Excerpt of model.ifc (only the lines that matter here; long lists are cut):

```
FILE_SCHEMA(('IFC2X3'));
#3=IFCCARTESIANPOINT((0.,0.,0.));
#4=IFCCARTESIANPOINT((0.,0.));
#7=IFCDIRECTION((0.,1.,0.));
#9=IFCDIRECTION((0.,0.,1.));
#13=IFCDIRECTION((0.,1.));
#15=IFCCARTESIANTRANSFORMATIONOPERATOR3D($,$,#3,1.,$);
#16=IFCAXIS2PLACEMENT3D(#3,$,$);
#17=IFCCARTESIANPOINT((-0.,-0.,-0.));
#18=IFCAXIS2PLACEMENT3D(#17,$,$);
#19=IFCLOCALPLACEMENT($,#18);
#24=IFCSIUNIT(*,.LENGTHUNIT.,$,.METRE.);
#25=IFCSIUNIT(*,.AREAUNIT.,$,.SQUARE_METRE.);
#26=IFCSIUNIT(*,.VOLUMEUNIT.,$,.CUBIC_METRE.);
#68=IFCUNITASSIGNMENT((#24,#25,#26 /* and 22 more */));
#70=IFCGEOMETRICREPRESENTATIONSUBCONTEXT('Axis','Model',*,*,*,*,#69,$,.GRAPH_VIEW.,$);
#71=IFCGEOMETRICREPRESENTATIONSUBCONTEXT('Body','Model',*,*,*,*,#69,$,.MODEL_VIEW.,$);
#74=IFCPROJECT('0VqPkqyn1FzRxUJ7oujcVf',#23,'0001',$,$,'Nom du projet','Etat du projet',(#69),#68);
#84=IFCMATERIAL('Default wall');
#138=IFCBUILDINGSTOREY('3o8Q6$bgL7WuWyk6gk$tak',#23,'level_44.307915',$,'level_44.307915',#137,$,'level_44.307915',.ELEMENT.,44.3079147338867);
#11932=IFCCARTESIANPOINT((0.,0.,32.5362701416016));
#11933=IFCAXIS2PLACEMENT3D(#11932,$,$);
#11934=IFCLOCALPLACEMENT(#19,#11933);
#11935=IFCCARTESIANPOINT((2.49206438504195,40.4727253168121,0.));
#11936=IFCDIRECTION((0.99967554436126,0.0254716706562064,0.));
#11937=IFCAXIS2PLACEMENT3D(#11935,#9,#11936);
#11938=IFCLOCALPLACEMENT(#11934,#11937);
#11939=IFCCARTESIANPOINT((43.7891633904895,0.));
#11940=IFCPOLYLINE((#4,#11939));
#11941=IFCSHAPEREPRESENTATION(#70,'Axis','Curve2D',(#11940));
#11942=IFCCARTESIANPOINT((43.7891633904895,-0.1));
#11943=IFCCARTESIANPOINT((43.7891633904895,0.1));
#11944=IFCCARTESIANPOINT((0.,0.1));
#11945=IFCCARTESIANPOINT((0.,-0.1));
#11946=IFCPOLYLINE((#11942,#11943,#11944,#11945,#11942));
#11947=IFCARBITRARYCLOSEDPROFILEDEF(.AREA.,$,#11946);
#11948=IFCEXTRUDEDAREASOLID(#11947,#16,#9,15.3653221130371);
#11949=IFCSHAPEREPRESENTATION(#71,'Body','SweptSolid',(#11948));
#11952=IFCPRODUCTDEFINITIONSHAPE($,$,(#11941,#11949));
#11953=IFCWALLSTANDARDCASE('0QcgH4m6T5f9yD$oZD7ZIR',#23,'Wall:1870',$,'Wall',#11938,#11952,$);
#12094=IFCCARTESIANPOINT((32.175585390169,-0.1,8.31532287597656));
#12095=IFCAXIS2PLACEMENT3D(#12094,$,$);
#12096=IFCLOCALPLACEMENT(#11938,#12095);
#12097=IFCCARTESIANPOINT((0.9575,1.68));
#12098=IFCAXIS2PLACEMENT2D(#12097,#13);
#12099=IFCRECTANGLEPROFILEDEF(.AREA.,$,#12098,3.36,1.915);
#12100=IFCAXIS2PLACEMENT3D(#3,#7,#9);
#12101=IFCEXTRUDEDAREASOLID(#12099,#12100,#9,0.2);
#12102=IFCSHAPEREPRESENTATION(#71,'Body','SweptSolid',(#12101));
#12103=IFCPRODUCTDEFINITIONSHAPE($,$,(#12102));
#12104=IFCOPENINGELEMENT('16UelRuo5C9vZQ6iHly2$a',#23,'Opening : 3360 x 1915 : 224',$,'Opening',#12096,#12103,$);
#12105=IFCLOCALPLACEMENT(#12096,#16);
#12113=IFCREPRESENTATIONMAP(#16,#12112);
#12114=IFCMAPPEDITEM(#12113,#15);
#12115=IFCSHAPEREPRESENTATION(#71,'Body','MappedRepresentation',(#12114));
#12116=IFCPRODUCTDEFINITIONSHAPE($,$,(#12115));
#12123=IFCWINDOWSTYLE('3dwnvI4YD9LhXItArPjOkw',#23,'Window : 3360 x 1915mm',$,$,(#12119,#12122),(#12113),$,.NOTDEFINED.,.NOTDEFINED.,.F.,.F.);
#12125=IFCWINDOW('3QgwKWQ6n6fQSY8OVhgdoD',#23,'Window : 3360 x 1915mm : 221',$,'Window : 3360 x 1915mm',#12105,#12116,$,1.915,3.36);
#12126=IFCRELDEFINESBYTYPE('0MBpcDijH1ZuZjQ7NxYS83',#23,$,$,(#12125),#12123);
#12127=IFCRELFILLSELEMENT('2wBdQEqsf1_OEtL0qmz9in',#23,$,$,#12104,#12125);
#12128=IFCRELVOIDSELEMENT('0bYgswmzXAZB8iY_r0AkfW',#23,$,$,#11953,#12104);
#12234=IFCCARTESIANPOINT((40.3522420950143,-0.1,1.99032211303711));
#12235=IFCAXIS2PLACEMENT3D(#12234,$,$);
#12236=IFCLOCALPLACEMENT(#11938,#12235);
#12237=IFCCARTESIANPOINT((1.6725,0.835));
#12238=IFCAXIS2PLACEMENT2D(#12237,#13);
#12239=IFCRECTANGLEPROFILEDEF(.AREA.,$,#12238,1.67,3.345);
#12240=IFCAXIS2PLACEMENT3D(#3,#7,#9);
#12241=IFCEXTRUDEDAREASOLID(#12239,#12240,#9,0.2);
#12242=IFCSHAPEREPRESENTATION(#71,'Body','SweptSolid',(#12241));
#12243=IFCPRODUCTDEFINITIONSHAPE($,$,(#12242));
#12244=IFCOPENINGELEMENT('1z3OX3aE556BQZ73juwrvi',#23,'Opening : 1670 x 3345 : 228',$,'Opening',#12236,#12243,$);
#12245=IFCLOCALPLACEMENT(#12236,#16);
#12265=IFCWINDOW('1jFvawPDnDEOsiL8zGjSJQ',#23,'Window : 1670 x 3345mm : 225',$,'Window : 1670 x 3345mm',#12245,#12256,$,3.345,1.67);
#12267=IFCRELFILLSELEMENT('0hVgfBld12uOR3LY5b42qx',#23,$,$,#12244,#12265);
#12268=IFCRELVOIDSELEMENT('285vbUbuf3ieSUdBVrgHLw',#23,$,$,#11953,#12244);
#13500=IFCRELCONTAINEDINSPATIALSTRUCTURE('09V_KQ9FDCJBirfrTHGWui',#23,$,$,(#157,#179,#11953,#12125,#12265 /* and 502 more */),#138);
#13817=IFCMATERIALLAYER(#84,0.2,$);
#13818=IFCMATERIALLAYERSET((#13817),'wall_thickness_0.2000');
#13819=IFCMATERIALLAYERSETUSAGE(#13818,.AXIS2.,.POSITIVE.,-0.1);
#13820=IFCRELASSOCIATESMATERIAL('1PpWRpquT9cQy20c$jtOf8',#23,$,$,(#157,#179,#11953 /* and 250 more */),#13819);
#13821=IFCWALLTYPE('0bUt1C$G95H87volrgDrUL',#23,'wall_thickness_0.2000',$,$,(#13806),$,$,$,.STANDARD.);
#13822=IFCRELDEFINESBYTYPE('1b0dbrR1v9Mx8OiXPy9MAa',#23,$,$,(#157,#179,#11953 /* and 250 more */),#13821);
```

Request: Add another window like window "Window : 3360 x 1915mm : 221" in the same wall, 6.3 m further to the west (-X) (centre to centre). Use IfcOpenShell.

```python
import ifcopenshell
import ifcopenshell.api.feature
import ifcopenshell.api.geometry
import ifcopenshell.api.root
import ifcopenshell.geom
import ifcopenshell.util.element
import ifcopenshell.util.placement
import ifcopenshell.util.shape

model = ifcopenshell.open("model.ifc")
settings = ifcopenshell.geom.settings()


def volume(element):
    """Net volume in cubic metres, openings subtracted."""
    shape = ifcopenshell.geom.create_shape(settings, element)
    return ifcopenshell.util.shape.get_volume(shape.geometry)


window = model.by_guid("3QgwKWQ6n6fQSY8OVhgdoD")
opening = window.FillsVoids[0].RelatingOpeningElement
wall = opening.VoidsElements[0].RelatingBuildingElement
before = volume(wall)
shift = ifcopenshell.util.placement.get_local_placement(wall.ObjectPlacement)[:3, 0] * -6.3

# copy_class copies the void relationship, type, container and properties, but no geometry.
new_opening = ifcopenshell.api.root.copy_class(model, product=opening)
new_opening.Representation = ifcopenshell.util.element.copy_deep(
    model, opening.Representation, exclude=["IfcGeometricRepresentationContext", "IfcRepresentationMap"]
)
new_opening.Name = "Opening : 3360 x 1915"
new_window = ifcopenshell.api.root.copy_class(model, product=window)
new_window.Representation = ifcopenshell.util.element.copy_deep(
    model, window.Representation, exclude=["IfcGeometricRepresentationContext", "IfcRepresentationMap"]
)
new_window.Name = "Window : 3360 x 1915mm"
fills = ifcopenshell.api.feature.add_filling(model, opening=new_opening, element=new_window)
fills.OwnerHistory = new_window.OwnerHistory  # required in IFC2X3

for old, new in ((opening, new_opening), (window, new_window)):
    matrix = ifcopenshell.util.placement.get_local_placement(old.ObjectPlacement)
    matrix[:3, 3] += shift
    ifcopenshell.api.geometry.edit_object_placement(model, product=new, matrix=matrix, is_si=False)

after = volume(wall)

print(f"wall volume {before:.3f} -> {after:.3f} m3")

model.write("model_edited.ifc")
```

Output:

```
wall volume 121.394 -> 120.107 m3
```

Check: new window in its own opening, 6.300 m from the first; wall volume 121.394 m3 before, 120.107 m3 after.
